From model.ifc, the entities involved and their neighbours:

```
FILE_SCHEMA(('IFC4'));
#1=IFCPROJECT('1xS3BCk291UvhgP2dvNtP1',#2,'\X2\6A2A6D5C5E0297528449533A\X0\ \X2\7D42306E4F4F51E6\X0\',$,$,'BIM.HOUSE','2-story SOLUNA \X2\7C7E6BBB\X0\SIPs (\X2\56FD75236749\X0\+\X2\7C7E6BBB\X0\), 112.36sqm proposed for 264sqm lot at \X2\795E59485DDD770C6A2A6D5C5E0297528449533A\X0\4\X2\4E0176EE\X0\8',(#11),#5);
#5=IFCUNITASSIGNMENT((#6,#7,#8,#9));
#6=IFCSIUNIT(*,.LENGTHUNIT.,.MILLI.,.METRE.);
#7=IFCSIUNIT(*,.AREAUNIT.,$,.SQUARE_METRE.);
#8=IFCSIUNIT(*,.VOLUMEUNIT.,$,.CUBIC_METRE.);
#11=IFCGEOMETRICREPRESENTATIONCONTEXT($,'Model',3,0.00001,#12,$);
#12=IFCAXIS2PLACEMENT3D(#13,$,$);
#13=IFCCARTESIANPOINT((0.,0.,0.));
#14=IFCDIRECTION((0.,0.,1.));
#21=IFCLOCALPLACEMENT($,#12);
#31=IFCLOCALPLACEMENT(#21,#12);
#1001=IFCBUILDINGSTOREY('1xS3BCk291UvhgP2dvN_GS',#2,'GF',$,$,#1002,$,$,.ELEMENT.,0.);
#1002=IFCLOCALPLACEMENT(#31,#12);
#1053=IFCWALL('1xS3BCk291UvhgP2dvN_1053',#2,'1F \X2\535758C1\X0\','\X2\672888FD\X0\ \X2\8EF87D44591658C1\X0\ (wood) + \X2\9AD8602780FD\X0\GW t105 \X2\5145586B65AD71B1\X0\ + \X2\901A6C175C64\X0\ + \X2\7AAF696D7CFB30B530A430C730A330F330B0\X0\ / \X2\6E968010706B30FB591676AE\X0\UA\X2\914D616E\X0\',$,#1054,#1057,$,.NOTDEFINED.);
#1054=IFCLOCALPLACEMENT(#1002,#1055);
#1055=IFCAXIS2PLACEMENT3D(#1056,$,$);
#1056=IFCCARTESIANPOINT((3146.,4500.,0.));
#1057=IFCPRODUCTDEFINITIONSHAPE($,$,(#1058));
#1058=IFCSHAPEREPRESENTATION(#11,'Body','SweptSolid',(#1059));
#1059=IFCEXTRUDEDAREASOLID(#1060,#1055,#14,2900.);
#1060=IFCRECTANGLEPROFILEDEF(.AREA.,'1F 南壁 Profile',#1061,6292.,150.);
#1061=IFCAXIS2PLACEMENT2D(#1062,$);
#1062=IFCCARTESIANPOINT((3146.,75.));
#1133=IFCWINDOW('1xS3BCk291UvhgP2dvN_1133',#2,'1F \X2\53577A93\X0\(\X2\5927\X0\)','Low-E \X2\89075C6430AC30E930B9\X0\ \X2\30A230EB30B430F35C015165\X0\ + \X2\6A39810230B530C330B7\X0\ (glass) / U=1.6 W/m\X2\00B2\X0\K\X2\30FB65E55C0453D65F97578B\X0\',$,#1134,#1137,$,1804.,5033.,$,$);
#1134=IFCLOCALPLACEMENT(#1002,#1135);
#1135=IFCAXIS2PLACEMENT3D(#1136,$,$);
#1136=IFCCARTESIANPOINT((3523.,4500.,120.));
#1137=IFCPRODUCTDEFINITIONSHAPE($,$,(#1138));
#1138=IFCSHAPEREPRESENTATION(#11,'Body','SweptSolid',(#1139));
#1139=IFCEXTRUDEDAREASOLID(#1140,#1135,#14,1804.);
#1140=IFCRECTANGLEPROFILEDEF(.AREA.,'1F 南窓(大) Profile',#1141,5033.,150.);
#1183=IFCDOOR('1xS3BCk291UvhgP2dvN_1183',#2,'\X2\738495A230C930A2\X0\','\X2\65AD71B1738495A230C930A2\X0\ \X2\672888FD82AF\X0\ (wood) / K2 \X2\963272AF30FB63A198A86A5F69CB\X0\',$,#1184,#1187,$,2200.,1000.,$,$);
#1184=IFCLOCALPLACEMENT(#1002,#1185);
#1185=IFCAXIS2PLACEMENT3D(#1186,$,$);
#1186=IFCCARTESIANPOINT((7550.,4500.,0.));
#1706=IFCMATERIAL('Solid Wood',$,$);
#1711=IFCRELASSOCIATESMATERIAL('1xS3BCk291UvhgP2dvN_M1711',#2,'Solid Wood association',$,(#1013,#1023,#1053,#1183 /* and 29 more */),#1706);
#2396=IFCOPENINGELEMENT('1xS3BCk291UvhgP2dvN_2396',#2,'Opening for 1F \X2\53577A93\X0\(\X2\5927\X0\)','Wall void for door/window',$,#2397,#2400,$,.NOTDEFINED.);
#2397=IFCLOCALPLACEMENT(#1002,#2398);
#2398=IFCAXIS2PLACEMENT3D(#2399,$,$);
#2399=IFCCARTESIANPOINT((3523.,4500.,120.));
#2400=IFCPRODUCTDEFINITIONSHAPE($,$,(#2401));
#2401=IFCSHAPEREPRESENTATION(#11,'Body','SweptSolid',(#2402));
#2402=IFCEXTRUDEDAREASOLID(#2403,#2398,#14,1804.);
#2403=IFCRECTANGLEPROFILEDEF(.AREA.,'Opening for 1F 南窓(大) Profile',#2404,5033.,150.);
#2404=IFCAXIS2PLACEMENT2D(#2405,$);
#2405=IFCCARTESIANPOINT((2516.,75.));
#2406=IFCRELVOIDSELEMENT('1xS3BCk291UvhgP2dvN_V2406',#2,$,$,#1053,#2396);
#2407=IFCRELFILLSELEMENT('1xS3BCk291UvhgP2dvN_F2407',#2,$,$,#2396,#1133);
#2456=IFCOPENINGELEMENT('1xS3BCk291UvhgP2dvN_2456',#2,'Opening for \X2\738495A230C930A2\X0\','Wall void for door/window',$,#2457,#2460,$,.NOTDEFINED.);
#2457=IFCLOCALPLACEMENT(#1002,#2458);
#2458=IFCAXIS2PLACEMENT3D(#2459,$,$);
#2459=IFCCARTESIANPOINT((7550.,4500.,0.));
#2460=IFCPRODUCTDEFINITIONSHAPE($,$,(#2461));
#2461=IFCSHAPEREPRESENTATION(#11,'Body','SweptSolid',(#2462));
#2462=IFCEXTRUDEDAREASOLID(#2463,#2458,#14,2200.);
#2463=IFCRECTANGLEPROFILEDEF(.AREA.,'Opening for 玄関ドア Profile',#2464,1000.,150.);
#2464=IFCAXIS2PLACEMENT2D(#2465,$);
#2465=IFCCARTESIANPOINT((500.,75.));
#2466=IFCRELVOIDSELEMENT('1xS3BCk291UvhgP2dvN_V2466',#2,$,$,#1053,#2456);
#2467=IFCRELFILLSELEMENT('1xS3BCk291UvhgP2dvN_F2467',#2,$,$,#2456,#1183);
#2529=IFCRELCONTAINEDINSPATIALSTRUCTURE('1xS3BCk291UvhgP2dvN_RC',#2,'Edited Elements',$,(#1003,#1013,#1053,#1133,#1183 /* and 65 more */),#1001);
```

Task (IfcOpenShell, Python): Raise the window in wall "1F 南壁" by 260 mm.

```python
import numpy as np
import ifcopenshell
import ifcopenshell.api.geometry
import ifcopenshell.util.placement
import ifcopenshell.util.unit

model = ifcopenshell.open("model.ifc")
unit_scale = ifcopenshell.util.unit.calculate_unit_scale(model)

window = model.by_guid("1xS3BCk291UvhgP2dvN_1133")
opening = window.FillsVoids[0].RelatingOpeningElement
dz = 260.0

shift = np.array([0.0, 0.0, dz])
# The window is not placed relative to its opening, so move both.
for product in (opening, window):
    matrix = ifcopenshell.util.placement.get_local_placement(product.ObjectPlacement)
    matrix[:3, 3] += shift
    ifcopenshell.api.geometry.edit_object_placement(model, product=product, matrix=matrix, is_si=False)

print(f"moved by {dz * unit_scale:+.3f} m")

model.write("model_rev.ifc")
```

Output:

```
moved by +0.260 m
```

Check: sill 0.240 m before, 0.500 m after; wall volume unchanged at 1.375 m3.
